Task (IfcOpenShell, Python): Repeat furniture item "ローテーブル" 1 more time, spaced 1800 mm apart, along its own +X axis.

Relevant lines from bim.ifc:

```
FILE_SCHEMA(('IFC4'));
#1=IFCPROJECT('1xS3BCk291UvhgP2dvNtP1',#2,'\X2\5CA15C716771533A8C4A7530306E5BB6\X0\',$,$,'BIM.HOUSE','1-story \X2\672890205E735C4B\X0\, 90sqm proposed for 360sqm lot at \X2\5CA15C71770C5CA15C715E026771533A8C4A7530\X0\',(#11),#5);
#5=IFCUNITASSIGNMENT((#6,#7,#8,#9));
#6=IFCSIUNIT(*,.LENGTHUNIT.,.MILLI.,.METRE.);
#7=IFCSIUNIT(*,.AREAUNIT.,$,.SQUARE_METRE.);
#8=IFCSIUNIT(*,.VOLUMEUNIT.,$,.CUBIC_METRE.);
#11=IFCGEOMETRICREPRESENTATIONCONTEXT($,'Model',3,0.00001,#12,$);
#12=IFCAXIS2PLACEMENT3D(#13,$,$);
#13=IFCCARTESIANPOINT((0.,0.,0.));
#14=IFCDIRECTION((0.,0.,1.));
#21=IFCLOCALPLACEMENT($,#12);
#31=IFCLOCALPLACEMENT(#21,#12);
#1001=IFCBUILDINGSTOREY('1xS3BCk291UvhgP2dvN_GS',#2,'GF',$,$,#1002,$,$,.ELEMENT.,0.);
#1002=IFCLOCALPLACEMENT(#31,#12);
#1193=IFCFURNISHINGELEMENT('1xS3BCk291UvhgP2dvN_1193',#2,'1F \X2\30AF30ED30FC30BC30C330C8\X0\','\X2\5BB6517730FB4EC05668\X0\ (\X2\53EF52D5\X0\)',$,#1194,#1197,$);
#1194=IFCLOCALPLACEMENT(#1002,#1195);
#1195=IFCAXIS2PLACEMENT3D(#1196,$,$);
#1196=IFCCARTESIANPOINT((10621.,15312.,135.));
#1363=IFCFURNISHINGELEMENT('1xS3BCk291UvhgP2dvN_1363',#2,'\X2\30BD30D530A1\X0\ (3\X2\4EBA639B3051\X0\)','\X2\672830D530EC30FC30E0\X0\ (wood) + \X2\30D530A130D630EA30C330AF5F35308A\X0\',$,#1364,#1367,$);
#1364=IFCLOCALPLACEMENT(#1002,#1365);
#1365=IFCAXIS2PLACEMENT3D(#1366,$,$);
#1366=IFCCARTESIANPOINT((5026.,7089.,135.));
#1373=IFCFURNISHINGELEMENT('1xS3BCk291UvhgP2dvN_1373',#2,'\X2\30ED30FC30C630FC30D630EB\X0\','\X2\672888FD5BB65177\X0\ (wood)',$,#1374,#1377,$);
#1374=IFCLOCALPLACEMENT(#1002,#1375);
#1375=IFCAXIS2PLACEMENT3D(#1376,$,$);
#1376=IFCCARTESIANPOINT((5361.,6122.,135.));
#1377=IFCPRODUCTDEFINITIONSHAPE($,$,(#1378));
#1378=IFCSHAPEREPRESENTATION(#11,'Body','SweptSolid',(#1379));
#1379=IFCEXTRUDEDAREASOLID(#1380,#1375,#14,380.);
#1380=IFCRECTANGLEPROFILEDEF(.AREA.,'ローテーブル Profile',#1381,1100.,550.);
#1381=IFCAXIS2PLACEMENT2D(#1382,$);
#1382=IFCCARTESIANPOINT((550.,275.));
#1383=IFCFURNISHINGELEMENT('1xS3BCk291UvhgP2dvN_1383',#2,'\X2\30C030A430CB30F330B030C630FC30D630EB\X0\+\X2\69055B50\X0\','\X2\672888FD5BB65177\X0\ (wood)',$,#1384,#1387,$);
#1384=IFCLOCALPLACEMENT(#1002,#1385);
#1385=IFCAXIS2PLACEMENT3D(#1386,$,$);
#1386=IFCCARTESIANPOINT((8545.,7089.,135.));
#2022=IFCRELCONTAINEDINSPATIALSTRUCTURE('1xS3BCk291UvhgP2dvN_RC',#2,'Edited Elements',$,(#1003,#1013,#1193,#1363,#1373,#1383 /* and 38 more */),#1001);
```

```python
import ifcopenshell
import ifcopenshell.api.geometry
import ifcopenshell.api.root
import ifcopenshell.util.element
import ifcopenshell.util.placement
import ifcopenshell.util.unit

model = ifcopenshell.open("bim.ifc")
unit_scale = ifcopenshell.util.unit.calculate_unit_scale(model)


def reuse_history(source, copy):
    """copy_class also copies each property set's owner history, people and application; keep the originals."""
    for rel in copy.IsDefinedBy:
        if rel.is_a("IfcRelDefinesByProperties") and (history := rel.RelatingPropertyDefinition.OwnerHistory):
            rel.RelatingPropertyDefinition.OwnerHistory = source.OwnerHistory
            ifcopenshell.util.element.remove_deep2(model, history)


source = model.by_guid("1xS3BCk291UvhgP2dvN_1373")
base = ifcopenshell.util.placement.get_local_placement(source.ObjectPlacement)
step = base[:3, 0] * 1.8 / unit_scale

for i in range(1, 2):
    copy = ifcopenshell.api.root.copy_class(model, product=source)
    copy.Representation = ifcopenshell.util.element.copy_deep(
        model, source.Representation, exclude=["IfcGeometricRepresentationContext", "IfcRepresentationMap"]
    )
    reuse_history(source, copy)
    matrix = base.copy()
    matrix[:3, 3] += i * step
    print("added at", matrix[:3, 3].round(3) + 0.0)
    ifcopenshell.api.geometry.edit_object_placement(model, product=copy, matrix=matrix, is_si=False)

model.write("bim-out.ifc")
```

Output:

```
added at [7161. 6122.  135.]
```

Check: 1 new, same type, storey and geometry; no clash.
